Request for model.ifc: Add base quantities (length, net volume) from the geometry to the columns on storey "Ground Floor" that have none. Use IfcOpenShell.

First a look at what the model holds.

```python
import ifcopenshell
import ifcopenshell.util.element
import ifcopenshell.util.unit

model = ifcopenshell.open("model.ifc")
print(model.schema)
for unit_type in ("LENGTHUNIT", "AREAUNIT", "VOLUMEUNIT"):
    print(unit_type, ifcopenshell.util.unit.calculate_unit_scale(model, unit_type))
storey = next(s for s in model.by_type("IfcBuildingStorey") if s.Name == "Ground Floor")
columns = [e for e in ifcopenshell.util.element.get_decomposition(storey) if e.is_a("IfcColumn")]
for e in sorted(columns, key=lambda e: e.id()):
    print(e.id(), e.is_a(), e.Name, list(ifcopenshell.util.element.get_psets(e, qtos_only=True)), sep=" | ")
```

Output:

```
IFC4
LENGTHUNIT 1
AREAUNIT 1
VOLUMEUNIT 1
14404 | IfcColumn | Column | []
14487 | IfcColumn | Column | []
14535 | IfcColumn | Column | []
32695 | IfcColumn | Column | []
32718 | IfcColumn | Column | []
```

```python
import ifcopenshell
import ifcopenshell.api.pset
import ifcopenshell.geom
import ifcopenshell.util.element
import ifcopenshell.util.shape
import ifcopenshell.util.unit

model = ifcopenshell.open("model.ifc")
unit_scale = ifcopenshell.util.unit.calculate_unit_scale(model)
volume_scale = ifcopenshell.util.unit.calculate_unit_scale(model, "VOLUMEUNIT")
settings = ifcopenshell.geom.settings()

storey = next(s for s in model.by_type("IfcBuildingStorey") if s.Name == "Ground Floor")
columns = [e for e in ifcopenshell.util.element.get_decomposition(storey) if e.is_a("IfcColumn")]

for e in sorted(columns, key=lambda e: e.id()):
    if ifcopenshell.util.element.get_psets(e, qtos_only=True, should_inherit=False):
        continue
    # Geometry comes back in metres, in the element's own axes.
    shape = ifcopenshell.geom.create_shape(settings, e)
    values = {
        "Length": ifcopenshell.util.shape.get_z(shape.geometry) / unit_scale,
        "NetVolume": ifcopenshell.util.shape.get_volume(shape.geometry) / volume_scale,
    }
    qto = ifcopenshell.api.pset.add_qto(model, product=e, name="Qto_ColumnBaseQuantities")
    ifcopenshell.api.pset.edit_qto(model, qto=qto, properties=values)
    print(e.id(), {k: round(v, 3) for k, v in values.items()})

model.write("model_updated.ifc")
```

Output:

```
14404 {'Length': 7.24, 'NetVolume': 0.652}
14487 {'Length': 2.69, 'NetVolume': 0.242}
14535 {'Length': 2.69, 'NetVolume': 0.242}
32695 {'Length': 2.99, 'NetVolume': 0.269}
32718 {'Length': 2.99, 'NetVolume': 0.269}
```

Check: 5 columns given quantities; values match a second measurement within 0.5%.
